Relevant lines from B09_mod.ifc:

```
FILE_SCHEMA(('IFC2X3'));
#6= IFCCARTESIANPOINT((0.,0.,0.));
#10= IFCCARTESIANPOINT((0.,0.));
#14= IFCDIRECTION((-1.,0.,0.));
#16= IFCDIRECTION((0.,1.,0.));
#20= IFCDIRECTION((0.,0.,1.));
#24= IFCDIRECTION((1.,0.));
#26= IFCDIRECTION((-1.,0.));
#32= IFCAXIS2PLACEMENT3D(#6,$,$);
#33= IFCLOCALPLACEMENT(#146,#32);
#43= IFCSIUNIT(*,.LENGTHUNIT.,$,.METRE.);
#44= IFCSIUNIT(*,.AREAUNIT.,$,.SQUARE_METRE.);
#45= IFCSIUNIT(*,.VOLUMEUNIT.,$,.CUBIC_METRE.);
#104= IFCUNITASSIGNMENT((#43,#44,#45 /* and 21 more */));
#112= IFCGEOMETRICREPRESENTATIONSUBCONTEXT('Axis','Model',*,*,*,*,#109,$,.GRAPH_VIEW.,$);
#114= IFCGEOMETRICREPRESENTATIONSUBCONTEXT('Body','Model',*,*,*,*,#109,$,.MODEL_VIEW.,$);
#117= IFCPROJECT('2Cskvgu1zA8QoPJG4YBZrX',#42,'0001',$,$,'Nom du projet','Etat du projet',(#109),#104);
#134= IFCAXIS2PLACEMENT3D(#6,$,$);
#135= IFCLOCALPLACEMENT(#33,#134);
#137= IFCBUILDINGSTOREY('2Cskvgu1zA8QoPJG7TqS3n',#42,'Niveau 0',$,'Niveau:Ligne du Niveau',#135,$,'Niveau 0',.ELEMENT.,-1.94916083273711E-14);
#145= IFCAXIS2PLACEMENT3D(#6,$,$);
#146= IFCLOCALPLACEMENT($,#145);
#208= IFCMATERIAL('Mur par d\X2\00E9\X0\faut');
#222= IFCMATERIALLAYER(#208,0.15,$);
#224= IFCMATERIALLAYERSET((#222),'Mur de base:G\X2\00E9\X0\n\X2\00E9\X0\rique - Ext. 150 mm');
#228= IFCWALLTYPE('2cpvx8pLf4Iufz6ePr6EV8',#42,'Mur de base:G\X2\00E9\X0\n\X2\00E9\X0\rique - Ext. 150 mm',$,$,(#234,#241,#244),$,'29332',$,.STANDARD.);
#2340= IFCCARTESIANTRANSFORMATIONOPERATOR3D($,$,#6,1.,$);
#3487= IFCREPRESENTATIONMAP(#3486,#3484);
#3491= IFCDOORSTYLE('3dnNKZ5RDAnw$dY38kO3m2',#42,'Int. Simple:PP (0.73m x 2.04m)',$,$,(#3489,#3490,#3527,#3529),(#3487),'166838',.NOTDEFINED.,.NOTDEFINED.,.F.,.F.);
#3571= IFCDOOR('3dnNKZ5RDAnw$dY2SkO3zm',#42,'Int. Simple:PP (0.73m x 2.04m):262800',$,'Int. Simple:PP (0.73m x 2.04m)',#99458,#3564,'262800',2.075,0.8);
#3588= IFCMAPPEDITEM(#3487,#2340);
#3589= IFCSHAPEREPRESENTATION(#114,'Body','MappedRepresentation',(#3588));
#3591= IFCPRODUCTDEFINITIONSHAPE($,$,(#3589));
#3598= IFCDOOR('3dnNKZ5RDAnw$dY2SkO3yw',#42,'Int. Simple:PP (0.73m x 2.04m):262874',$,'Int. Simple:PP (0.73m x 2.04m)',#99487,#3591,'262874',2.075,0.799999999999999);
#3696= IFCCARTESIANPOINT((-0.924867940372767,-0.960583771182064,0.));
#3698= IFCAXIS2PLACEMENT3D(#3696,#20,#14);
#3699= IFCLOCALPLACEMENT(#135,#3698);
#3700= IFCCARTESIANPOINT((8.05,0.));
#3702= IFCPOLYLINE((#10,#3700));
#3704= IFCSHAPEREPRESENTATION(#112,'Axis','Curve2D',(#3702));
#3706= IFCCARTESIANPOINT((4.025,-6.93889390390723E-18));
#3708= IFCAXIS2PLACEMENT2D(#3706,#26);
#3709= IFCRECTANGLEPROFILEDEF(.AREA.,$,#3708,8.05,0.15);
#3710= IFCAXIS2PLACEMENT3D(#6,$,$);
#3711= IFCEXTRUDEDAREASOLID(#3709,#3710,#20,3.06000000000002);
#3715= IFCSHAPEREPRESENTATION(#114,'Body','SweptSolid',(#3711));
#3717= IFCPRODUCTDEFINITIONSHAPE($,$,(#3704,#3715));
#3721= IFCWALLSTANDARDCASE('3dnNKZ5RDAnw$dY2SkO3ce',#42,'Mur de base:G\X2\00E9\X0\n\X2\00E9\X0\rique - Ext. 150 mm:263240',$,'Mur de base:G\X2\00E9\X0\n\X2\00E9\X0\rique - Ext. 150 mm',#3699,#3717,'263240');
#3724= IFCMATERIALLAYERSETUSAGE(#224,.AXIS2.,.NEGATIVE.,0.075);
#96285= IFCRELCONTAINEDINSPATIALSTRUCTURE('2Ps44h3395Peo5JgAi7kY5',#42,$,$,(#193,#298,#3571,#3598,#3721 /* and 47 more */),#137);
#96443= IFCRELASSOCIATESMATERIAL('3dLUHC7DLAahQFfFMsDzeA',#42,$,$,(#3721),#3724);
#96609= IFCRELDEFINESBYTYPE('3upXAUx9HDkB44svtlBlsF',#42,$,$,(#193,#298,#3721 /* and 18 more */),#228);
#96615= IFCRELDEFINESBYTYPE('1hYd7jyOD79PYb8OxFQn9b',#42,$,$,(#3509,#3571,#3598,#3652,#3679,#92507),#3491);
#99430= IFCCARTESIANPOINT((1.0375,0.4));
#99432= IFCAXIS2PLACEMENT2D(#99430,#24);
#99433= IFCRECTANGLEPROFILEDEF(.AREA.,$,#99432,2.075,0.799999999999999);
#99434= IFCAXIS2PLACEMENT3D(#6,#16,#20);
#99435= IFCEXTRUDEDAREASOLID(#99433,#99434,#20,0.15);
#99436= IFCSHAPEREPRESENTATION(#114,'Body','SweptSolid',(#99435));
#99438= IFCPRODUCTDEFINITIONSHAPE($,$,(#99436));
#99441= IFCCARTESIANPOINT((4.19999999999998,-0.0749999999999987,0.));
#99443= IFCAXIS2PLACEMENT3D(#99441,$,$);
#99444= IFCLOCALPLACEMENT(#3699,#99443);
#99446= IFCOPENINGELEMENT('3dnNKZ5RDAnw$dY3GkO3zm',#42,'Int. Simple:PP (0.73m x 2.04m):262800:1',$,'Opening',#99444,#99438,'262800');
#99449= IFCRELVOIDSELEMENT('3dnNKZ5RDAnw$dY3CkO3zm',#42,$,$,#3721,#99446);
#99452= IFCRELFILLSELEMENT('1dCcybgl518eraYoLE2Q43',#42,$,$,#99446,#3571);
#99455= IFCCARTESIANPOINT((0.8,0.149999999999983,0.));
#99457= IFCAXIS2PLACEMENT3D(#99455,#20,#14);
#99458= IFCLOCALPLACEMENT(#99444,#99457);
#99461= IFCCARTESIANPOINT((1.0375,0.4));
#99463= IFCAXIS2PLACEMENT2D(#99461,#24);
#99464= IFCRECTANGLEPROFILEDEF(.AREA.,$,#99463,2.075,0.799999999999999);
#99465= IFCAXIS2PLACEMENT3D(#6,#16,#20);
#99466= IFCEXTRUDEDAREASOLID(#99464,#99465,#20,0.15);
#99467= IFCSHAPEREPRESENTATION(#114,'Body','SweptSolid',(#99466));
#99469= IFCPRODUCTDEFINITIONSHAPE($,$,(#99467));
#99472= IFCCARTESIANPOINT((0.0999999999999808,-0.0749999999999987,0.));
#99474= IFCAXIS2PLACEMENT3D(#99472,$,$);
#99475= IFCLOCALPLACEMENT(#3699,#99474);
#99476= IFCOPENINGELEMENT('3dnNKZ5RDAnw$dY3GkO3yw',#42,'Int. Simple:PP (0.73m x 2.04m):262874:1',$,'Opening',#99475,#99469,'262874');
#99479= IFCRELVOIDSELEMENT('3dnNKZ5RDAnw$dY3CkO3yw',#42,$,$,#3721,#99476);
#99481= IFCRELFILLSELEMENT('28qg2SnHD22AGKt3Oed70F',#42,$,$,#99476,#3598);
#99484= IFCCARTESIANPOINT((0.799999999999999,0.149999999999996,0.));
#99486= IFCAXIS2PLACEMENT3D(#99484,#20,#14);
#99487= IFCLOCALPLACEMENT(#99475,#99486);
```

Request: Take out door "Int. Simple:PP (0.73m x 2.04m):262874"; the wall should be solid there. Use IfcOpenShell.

```python
import ifcopenshell
import ifcopenshell.api.feature
import ifcopenshell.api.root
import ifcopenshell.geom
import ifcopenshell.util.shape

model = ifcopenshell.open("B09_mod.ifc")
settings = ifcopenshell.geom.settings()


def volume(element):
    """Net volume in cubic metres, openings subtracted."""
    shape = ifcopenshell.geom.create_shape(settings, element)
    return ifcopenshell.util.shape.get_volume(shape.geometry)


door = model.by_id(3598)
opening = door.FillsVoids[0].RelatingOpeningElement
wall = opening.VoidsElements[0].RelatingBuildingElement
before = volume(wall)

ifcopenshell.api.root.remove_product(model, product=door)
ifcopenshell.api.feature.remove_feature(model, feature=opening)

after = volume(wall)

print(f"wall volume {before:.3f} -> {after:.3f} m3")

model.write("B09_mod_rev.ifc")
```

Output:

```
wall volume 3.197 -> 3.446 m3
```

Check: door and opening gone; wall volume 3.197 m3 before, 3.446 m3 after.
